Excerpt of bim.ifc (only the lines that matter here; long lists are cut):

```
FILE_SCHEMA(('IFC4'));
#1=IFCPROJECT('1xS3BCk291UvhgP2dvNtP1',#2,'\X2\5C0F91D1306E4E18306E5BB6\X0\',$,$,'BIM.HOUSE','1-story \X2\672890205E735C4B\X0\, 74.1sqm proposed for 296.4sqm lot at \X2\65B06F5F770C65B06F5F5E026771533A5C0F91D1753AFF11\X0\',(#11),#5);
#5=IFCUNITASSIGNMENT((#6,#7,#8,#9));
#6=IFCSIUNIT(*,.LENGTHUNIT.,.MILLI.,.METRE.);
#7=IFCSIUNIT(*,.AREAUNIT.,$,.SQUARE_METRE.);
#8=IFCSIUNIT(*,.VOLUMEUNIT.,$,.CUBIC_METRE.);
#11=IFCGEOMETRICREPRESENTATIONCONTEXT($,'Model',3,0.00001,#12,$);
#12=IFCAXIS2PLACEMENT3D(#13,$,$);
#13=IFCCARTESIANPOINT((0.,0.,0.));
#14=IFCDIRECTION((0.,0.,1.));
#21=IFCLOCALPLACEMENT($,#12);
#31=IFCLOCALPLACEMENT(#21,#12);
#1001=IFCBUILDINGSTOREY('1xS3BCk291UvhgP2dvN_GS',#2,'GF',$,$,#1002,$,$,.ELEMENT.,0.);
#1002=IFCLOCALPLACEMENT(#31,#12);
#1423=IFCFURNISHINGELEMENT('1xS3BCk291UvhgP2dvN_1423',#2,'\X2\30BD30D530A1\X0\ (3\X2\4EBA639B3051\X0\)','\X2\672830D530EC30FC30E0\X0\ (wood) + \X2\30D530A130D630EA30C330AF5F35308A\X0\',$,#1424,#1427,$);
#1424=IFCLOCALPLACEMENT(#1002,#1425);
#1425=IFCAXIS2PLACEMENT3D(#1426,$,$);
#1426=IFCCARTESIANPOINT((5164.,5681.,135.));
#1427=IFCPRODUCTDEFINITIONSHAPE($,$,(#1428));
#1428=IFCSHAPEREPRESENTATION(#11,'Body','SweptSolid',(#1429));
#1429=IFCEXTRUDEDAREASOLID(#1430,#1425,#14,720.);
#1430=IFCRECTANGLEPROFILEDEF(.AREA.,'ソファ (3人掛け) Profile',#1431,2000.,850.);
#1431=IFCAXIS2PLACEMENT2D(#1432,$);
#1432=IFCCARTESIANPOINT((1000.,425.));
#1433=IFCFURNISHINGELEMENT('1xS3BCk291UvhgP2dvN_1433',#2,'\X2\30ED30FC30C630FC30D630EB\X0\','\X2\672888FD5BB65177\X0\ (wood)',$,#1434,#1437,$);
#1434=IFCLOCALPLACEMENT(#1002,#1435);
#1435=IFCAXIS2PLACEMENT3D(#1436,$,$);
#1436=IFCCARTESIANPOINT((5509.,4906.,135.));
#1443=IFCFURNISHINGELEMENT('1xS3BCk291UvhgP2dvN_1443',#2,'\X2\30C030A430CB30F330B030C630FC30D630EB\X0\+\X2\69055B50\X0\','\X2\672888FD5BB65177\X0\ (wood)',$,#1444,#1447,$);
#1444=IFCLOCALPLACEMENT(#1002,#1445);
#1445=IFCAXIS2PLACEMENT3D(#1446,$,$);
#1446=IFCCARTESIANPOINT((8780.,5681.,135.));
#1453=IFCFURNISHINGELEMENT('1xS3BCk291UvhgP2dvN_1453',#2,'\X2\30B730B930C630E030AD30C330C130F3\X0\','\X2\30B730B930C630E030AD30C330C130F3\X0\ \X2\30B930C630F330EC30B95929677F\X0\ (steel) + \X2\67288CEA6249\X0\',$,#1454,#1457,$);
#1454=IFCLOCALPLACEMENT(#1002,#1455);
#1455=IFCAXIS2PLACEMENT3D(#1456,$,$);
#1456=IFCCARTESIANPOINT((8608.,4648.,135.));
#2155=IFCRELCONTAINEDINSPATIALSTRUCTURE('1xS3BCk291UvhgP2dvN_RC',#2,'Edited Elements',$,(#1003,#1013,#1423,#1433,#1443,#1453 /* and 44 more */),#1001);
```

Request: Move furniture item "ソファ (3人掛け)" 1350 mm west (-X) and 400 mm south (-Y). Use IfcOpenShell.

```python
import ifcopenshell
import ifcopenshell.api.geometry
import ifcopenshell.util.placement
import ifcopenshell.util.unit

model = ifcopenshell.open("bim.ifc")
unit_scale = ifcopenshell.util.unit.calculate_unit_scale(model)

item = model.by_guid("1xS3BCk291UvhgP2dvN_1423")
matrix = ifcopenshell.util.placement.get_local_placement(item.ObjectPlacement)
matrix[0, 3] -= 1.35 / unit_scale
matrix[1, 3] -= 0.4 / unit_scale
ifcopenshell.api.geometry.edit_object_placement(model, product=item, matrix=matrix, is_si=False)

print(ifcopenshell.util.placement.get_local_placement(item.ObjectPlacement).round(3) + 0.0)

model.write("bim_updated.ifc")
```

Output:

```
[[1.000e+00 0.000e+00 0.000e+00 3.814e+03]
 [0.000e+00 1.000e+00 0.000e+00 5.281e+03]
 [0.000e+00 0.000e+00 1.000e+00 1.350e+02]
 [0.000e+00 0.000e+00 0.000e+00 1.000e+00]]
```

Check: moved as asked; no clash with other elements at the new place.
